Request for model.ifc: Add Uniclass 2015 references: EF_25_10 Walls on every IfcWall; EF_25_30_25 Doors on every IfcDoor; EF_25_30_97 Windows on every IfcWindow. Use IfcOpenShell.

First a look at what the model holds.

```python
import ifcopenshell

model = ifcopenshell.open("model.ifc")
print(model.schema)
print("classifications:", [c.Name for c in model.by_type("IfcClassification")])
for ifc_class in ("IfcDoor", "IfcRoof", "IfcStair", "IfcWall", "IfcWindow"):
    print(ifc_class, len(model.by_type(ifc_class)))
```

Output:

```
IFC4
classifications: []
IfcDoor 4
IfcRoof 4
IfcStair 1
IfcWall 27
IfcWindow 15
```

```python
import ifcopenshell
import ifcopenshell.api.classification

model = ifcopenshell.open("model.ifc")

system = ifcopenshell.api.classification.add_classification(model, classification="Uniclass 2015")

codes = {
    "IfcWall": ("EF_25_10", "Walls"),
    "IfcDoor": ("EF_25_30_25", "Doors"),
    "IfcWindow": ("EF_25_30_97", "Windows"),
}
for ifc_class, (code, name) in codes.items():
    products = model.by_type(ifc_class)
    ifcopenshell.api.classification.add_reference(
        model, products=products, classification=system, identification=code, name=name
    )
    print(code, len(products))

model.write("model_edited.ifc")
```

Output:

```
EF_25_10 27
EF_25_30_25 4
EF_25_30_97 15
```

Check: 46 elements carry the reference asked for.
